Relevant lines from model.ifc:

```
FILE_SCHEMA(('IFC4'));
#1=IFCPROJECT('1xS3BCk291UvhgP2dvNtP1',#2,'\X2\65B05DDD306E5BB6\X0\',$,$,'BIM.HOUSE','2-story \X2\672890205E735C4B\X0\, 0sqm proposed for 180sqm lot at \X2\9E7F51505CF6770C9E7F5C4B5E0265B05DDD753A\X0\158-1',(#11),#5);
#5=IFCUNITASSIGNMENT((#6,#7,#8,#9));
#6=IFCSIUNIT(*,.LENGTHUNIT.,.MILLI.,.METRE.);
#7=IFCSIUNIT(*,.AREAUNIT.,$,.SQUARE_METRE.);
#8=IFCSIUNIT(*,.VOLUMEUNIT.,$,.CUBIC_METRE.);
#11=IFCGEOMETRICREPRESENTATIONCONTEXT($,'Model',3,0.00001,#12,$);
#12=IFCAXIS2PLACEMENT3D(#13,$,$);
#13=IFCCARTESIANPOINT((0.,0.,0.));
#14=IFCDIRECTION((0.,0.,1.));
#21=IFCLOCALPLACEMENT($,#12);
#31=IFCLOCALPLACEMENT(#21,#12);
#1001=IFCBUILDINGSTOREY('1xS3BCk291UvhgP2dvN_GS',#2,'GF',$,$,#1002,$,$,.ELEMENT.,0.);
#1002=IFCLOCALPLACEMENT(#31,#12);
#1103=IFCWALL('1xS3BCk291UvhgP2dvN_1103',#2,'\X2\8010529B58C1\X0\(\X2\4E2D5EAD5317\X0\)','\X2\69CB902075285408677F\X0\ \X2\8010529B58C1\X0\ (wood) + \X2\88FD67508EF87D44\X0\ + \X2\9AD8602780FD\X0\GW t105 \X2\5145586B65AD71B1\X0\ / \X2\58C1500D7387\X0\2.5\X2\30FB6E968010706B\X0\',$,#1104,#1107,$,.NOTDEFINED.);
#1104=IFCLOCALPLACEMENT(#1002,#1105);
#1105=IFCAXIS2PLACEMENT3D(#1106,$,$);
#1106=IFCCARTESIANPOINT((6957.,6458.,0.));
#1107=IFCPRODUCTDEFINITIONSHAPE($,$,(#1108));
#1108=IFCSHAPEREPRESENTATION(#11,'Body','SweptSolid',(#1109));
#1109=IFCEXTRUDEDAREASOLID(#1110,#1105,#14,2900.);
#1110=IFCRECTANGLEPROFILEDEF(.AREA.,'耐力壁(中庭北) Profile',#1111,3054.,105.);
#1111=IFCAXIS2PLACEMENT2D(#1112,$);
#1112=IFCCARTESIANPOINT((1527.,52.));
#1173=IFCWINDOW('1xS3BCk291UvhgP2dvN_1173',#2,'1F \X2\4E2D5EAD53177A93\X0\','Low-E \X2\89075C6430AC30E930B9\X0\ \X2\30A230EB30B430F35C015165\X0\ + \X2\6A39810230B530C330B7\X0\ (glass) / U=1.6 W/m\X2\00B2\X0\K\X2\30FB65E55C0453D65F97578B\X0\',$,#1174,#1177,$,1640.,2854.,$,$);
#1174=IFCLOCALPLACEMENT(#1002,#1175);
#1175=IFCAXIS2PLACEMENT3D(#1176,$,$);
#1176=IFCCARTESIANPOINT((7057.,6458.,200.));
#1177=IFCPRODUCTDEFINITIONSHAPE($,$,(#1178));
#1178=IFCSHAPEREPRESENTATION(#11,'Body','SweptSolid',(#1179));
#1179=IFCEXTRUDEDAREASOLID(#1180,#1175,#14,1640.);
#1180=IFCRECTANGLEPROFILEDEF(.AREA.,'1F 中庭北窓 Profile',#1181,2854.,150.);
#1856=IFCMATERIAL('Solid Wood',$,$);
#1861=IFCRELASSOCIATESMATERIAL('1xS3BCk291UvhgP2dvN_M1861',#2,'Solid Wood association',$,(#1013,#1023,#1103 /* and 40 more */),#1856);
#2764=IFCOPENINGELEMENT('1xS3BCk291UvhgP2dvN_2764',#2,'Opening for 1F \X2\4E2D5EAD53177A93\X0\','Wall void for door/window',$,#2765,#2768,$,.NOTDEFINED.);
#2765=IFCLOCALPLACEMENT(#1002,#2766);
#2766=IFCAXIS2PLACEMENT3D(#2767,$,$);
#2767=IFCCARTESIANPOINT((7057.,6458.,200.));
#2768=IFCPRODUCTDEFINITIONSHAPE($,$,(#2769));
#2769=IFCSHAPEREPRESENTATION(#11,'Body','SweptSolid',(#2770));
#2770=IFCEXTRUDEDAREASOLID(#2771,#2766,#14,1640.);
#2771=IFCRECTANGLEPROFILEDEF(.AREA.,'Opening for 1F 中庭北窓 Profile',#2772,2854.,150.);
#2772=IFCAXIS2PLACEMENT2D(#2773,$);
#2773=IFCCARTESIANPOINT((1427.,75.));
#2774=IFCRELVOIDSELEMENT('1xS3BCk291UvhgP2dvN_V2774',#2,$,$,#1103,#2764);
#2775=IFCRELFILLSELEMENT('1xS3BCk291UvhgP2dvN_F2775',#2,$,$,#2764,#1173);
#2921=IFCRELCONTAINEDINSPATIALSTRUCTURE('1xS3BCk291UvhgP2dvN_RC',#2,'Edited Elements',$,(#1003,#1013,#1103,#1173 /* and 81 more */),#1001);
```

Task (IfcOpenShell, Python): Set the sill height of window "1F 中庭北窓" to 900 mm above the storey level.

```python
import numpy as np
import ifcopenshell
import ifcopenshell.api.geometry
import ifcopenshell.geom
import ifcopenshell.util.element
import ifcopenshell.util.placement
import ifcopenshell.util.shape
import ifcopenshell.util.unit

model = ifcopenshell.open("model.ifc")
unit_scale = ifcopenshell.util.unit.calculate_unit_scale(model)

window = model.by_id(1173)
opening = window.FillsVoids[0].RelatingOpeningElement
storey = ifcopenshell.util.element.get_container(window, ifc_class="IfcBuildingStorey")
level = ifcopenshell.util.placement.get_local_placement(storey.ObjectPlacement)[2, 3]

# The opening's origin need not be at the sill, so measure its lowest point.
shape = ifcopenshell.geom.create_shape(ifcopenshell.geom.settings(), opening)
bottom = ifcopenshell.util.shape.get_shape_bottom_elevation(shape, shape.geometry) / unit_scale
dz = level + 0.9 / unit_scale - bottom

shift = np.array([0.0, 0.0, dz])
# The window is not placed relative to its opening, so move both.
for product in (opening, window):
    matrix = ifcopenshell.util.placement.get_local_placement(product.ObjectPlacement)
    matrix[:3, 3] += shift
    ifcopenshell.api.geometry.edit_object_placement(model, product=product, matrix=matrix, is_si=False)

print(f"moved by {dz * unit_scale:+.3f} m")

model.write("model_v2.ifc")
```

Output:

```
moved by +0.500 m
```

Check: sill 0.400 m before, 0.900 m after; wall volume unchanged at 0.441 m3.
